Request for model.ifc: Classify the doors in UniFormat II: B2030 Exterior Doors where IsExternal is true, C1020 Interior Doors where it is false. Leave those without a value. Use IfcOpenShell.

First a look at what the model holds.

```python
import ifcopenshell
import ifcopenshell.util.element

model = ifcopenshell.open("model.ifc")
print(model.schema)
print("classifications:", [c.Name for c in model.by_type("IfcClassification")])
values = [ifcopenshell.util.element.get_pset(e, "Pset_DoorCommon", "IsExternal") for e in model.by_type("IfcDoor")]
for value in (True, False, None):
    print("IsExternal", value, values.count(value))
```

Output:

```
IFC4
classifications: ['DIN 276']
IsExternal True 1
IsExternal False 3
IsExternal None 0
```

```python
import ifcopenshell
import ifcopenshell.api.classification
import ifcopenshell.util.element

model = ifcopenshell.open("model.ifc")

system = ifcopenshell.api.classification.add_classification(model, classification="UniFormat II")

doors = model.by_type("IfcDoor")
external = {e: ifcopenshell.util.element.get_pset(e, "Pset_DoorCommon", "IsExternal") for e in doors}
for flag, code, name in ((True, "B2030", "Exterior Doors"), (False, "C1020", "Interior Doors")):
    products = [e for e in doors if external[e] is flag]
    ifcopenshell.api.classification.add_reference(
        model, products=products, classification=system, identification=code, name=name
    )
    print(code, len(products))

model.write("model_v2.ifc")
```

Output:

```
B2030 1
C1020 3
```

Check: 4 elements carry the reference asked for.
